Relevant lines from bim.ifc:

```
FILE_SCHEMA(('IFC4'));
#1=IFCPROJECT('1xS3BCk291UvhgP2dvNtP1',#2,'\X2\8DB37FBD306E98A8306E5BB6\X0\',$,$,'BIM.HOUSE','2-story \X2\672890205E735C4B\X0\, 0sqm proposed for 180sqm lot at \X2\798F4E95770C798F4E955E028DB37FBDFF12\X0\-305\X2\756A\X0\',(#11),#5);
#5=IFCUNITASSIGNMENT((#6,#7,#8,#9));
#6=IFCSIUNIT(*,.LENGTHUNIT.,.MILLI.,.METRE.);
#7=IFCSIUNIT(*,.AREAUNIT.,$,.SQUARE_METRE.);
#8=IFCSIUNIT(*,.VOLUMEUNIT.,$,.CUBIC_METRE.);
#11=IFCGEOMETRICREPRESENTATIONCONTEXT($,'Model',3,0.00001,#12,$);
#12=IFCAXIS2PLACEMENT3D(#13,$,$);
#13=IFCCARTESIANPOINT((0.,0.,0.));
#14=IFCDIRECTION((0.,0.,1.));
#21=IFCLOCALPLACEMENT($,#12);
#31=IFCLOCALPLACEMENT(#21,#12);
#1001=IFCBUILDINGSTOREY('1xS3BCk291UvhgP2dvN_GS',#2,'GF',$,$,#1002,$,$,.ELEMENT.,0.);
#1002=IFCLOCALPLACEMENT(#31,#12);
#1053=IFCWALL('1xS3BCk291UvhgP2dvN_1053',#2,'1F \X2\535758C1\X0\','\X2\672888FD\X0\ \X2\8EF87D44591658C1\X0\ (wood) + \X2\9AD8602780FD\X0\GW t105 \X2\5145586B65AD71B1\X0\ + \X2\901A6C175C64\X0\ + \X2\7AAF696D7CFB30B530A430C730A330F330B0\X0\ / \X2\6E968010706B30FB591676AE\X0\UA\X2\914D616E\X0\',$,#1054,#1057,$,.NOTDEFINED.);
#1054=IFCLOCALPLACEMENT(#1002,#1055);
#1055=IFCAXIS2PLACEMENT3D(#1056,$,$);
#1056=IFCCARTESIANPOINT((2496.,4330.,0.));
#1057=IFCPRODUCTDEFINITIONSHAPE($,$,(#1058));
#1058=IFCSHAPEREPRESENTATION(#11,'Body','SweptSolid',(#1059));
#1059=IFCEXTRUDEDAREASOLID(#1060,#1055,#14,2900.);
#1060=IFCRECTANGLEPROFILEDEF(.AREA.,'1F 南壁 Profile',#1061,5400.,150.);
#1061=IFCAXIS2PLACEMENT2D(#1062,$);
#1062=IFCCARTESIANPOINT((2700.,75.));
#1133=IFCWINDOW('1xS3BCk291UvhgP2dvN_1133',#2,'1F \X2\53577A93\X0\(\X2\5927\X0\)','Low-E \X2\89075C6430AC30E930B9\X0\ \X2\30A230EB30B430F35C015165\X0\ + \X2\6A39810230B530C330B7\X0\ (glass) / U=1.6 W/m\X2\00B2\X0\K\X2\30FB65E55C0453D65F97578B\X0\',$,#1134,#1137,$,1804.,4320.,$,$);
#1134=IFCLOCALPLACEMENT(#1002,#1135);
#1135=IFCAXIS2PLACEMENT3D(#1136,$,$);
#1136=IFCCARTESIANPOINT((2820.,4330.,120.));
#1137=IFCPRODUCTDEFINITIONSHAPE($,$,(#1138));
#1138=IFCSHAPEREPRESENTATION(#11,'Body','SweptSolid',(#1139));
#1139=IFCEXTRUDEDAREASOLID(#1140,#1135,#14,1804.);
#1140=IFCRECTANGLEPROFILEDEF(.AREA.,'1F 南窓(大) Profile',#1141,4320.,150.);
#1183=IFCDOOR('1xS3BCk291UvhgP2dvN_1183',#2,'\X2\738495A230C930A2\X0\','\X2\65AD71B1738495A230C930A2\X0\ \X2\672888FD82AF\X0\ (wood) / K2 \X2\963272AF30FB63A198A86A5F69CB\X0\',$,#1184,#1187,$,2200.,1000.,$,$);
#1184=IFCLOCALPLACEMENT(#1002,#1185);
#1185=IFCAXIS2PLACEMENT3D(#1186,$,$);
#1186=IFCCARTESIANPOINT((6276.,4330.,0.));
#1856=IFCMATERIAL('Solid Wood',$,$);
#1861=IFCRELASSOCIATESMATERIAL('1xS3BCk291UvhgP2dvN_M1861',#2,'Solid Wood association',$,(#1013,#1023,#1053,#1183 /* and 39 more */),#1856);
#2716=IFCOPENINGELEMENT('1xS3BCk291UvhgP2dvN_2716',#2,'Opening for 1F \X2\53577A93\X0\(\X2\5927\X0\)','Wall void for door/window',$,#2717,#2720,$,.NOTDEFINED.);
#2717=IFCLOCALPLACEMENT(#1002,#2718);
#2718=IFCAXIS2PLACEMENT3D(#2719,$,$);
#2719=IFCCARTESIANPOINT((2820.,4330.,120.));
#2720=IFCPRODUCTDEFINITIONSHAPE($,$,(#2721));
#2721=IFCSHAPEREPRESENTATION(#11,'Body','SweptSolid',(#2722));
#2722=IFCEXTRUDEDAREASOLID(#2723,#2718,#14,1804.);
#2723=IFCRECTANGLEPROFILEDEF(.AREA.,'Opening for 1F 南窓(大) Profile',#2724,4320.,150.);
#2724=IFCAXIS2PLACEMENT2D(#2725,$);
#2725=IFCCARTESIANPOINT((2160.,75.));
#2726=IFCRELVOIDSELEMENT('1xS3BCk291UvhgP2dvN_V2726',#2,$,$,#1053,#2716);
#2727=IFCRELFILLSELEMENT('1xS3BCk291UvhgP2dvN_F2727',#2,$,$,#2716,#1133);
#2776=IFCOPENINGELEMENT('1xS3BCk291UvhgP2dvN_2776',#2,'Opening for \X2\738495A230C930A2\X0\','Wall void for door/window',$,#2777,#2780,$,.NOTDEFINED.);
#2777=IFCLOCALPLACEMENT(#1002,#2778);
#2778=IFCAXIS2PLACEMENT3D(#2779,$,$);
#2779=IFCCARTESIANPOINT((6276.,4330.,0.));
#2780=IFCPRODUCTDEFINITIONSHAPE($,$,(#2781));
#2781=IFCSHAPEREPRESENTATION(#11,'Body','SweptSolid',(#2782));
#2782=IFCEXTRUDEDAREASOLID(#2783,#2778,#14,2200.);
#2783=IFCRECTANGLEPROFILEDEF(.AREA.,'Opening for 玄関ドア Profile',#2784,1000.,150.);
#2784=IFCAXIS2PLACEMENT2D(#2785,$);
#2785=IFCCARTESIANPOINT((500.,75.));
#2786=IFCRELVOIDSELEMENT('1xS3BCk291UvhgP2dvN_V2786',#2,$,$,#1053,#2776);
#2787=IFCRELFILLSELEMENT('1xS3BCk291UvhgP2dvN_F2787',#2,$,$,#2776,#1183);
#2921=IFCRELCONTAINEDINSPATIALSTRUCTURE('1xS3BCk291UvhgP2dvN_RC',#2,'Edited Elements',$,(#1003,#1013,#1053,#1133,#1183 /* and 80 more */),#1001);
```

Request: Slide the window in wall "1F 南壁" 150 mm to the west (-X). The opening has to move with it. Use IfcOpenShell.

```python
import ifcopenshell
import ifcopenshell.api.geometry
import ifcopenshell.util.placement
import ifcopenshell.util.unit

model = ifcopenshell.open("bim.ifc")
unit_scale = ifcopenshell.util.unit.calculate_unit_scale(model)

window = model.by_guid("1xS3BCk291UvhgP2dvN_1133")
opening = window.FillsVoids[0].RelatingOpeningElement
wall = opening.VoidsElements[0].RelatingBuildingElement

wall_matrix = ifcopenshell.util.placement.get_local_placement(wall.ObjectPlacement)
shift = wall_matrix[:3, 0] * -0.15 / unit_scale
before = ifcopenshell.util.placement.get_local_placement(window.ObjectPlacement)[:3, 3].copy()

# The window is not placed relative to its opening, so move both.
for product in (opening, window):
    matrix = ifcopenshell.util.placement.get_local_placement(product.ObjectPlacement)
    matrix[:3, 3] += shift
    ifcopenshell.api.geometry.edit_object_placement(model, product=product, matrix=matrix, is_si=False)

after = ifcopenshell.util.placement.get_local_placement(window.ObjectPlacement)[:3, 3]
print("window moved by", (after - before).round(3) + 0.0)

model.write("bim_v2.ifc")
```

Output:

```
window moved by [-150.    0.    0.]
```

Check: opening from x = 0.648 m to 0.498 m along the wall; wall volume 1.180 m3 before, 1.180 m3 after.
